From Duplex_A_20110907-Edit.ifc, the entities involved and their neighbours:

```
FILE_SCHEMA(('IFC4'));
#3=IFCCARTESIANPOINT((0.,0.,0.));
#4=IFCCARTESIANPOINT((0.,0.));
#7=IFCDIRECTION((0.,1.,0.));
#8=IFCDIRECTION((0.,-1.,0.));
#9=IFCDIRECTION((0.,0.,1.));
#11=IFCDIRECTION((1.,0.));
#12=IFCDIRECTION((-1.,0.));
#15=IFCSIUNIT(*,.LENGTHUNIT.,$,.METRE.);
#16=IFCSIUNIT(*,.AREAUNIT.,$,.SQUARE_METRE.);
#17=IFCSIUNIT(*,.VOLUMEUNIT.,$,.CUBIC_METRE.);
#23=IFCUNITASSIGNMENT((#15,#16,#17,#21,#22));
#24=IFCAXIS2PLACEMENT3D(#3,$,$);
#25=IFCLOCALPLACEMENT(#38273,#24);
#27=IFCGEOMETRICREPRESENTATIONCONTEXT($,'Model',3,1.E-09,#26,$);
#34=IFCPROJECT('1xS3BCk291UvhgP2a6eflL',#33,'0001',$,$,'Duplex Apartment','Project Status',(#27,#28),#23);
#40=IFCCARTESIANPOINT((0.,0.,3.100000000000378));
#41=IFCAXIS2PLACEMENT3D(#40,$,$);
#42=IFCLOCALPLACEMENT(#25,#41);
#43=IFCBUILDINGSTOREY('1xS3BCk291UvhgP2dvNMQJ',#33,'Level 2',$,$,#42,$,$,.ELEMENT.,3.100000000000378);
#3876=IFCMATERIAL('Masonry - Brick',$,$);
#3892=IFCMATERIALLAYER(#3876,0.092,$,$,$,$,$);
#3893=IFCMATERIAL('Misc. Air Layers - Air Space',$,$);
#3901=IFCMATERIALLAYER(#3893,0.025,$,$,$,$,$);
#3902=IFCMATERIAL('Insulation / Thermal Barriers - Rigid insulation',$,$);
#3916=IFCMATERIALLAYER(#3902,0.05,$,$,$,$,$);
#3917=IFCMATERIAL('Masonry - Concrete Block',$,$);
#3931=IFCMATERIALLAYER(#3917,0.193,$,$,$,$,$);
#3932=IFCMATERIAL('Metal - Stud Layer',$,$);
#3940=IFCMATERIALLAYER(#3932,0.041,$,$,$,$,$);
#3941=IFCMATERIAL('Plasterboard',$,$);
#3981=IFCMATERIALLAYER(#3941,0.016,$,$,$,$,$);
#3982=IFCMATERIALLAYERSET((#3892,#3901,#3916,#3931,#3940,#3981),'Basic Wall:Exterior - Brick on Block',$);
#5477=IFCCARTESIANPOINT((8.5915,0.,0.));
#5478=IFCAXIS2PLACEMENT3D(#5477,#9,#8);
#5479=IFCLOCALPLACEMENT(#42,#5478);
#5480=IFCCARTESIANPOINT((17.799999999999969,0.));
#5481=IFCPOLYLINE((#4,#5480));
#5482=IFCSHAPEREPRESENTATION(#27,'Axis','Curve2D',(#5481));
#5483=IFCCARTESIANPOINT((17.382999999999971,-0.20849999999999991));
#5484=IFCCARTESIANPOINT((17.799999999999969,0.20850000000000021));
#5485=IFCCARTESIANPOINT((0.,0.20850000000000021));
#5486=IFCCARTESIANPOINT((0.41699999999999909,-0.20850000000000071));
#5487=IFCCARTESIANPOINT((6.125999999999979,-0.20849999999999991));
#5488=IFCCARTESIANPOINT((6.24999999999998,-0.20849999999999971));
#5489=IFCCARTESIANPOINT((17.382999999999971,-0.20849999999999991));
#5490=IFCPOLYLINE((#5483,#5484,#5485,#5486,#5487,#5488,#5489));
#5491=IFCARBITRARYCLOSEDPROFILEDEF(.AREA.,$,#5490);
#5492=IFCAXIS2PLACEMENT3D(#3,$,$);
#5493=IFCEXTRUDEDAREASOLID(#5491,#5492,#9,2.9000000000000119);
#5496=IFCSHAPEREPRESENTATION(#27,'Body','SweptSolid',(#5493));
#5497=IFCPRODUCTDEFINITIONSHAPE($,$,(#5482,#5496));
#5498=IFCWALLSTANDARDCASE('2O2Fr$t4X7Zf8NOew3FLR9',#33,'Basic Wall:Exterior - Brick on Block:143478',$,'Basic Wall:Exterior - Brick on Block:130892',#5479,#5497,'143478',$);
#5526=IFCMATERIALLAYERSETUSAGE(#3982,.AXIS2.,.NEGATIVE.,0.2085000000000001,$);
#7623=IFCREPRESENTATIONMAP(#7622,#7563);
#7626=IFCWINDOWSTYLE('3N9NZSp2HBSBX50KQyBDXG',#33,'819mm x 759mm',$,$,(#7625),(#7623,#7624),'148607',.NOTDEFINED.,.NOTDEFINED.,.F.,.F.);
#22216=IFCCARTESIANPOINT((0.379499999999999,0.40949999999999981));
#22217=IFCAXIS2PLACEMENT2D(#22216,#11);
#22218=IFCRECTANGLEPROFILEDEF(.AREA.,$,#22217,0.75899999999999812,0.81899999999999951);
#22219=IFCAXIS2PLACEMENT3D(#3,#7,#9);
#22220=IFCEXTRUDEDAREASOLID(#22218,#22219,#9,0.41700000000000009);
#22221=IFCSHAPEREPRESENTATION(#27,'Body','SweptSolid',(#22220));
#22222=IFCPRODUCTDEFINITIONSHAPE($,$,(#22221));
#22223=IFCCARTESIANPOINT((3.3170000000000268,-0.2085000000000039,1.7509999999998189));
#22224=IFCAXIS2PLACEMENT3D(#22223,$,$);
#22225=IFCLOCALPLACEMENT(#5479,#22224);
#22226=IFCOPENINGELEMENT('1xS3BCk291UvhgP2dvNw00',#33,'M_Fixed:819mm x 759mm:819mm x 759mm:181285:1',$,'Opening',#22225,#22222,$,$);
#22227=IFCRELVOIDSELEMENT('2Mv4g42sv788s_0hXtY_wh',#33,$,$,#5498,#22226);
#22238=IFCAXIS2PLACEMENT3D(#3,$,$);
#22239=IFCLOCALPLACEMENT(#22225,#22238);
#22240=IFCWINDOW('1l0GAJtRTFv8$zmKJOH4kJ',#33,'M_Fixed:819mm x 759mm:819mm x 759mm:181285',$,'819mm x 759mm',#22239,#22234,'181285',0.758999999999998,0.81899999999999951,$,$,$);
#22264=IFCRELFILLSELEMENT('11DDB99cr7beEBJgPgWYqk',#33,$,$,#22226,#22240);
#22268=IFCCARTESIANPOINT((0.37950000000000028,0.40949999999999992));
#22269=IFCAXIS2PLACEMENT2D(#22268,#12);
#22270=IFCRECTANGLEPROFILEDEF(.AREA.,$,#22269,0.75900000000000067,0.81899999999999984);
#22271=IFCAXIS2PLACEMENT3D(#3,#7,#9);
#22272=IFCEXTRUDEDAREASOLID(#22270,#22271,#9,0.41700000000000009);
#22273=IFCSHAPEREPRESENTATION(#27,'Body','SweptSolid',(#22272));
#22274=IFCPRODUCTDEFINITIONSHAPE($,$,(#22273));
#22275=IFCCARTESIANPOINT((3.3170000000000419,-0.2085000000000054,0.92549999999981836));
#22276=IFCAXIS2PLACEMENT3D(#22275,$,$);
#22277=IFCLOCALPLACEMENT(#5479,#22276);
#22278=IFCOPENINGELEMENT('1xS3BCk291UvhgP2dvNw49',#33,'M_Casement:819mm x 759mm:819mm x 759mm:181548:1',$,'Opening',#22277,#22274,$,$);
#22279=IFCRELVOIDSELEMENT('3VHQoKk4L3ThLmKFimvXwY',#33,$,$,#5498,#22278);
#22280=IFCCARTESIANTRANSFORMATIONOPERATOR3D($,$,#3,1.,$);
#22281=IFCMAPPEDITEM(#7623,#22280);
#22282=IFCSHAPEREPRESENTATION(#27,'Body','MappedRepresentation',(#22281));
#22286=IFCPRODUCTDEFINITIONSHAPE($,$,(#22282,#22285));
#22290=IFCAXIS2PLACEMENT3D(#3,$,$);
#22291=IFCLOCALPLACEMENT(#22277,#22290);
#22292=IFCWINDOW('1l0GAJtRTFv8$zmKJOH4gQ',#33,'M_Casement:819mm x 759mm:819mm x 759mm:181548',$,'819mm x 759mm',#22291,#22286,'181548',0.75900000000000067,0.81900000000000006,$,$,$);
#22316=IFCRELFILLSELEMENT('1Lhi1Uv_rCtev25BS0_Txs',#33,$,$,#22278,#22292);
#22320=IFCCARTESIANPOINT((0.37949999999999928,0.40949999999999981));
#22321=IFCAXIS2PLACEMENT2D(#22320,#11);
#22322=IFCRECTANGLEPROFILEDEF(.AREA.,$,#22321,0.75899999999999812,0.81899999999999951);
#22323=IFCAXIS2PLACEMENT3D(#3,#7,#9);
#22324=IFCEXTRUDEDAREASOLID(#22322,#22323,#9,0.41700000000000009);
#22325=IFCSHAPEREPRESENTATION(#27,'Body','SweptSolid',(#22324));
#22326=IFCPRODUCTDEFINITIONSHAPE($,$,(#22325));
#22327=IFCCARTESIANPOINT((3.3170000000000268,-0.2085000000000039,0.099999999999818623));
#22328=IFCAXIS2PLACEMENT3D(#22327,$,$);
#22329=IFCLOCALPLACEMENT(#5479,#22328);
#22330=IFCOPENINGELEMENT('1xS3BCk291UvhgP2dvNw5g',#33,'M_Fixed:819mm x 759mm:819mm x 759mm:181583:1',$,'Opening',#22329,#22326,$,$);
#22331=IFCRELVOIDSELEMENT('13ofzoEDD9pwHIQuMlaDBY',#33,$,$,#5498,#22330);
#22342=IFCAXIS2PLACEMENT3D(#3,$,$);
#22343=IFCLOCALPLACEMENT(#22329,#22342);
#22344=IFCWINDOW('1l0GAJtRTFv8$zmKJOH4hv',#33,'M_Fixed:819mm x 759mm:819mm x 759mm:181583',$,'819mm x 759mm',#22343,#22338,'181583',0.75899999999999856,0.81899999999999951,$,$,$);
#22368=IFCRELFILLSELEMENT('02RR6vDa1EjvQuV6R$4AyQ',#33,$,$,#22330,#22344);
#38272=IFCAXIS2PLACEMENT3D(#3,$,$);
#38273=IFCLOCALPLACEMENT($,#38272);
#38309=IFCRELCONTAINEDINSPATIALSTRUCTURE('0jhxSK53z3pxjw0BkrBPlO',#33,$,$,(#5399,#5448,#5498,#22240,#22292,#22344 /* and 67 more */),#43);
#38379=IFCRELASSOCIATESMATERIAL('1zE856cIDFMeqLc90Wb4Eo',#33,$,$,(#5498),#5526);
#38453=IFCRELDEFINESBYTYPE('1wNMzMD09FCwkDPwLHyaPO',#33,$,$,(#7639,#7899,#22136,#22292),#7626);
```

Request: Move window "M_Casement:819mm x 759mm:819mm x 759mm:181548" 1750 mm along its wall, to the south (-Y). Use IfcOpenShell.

```python
import ifcopenshell
import ifcopenshell.api.geometry
import ifcopenshell.util.placement
import ifcopenshell.util.unit

model = ifcopenshell.open("Duplex_A_20110907-Edit.ifc")
unit_scale = ifcopenshell.util.unit.calculate_unit_scale(model)

window = model.by_guid("1l0GAJtRTFv8$zmKJOH4gQ")
opening = window.FillsVoids[0].RelatingOpeningElement
wall = opening.VoidsElements[0].RelatingBuildingElement

wall_matrix = ifcopenshell.util.placement.get_local_placement(wall.ObjectPlacement)
shift = wall_matrix[:3, 0] * 1.75 / unit_scale
before = ifcopenshell.util.placement.get_local_placement(window.ObjectPlacement)[:3, 3].copy()

# The window is placed relative to its opening, so it follows when the opening moves.
matrix = ifcopenshell.util.placement.get_local_placement(opening.ObjectPlacement)
matrix[:3, 3] += shift
ifcopenshell.api.geometry.edit_object_placement(
    model, product=opening, matrix=matrix, is_si=False, should_transform_children=True
)

after = ifcopenshell.util.placement.get_local_placement(window.ObjectPlacement)[:3, 3]
print("window moved by", (after - before).round(3) + 0.0)

model.write("Duplex_A_20110907-Edit_v2.ifc")
```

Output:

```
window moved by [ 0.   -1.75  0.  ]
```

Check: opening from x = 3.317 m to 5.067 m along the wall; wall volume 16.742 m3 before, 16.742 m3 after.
